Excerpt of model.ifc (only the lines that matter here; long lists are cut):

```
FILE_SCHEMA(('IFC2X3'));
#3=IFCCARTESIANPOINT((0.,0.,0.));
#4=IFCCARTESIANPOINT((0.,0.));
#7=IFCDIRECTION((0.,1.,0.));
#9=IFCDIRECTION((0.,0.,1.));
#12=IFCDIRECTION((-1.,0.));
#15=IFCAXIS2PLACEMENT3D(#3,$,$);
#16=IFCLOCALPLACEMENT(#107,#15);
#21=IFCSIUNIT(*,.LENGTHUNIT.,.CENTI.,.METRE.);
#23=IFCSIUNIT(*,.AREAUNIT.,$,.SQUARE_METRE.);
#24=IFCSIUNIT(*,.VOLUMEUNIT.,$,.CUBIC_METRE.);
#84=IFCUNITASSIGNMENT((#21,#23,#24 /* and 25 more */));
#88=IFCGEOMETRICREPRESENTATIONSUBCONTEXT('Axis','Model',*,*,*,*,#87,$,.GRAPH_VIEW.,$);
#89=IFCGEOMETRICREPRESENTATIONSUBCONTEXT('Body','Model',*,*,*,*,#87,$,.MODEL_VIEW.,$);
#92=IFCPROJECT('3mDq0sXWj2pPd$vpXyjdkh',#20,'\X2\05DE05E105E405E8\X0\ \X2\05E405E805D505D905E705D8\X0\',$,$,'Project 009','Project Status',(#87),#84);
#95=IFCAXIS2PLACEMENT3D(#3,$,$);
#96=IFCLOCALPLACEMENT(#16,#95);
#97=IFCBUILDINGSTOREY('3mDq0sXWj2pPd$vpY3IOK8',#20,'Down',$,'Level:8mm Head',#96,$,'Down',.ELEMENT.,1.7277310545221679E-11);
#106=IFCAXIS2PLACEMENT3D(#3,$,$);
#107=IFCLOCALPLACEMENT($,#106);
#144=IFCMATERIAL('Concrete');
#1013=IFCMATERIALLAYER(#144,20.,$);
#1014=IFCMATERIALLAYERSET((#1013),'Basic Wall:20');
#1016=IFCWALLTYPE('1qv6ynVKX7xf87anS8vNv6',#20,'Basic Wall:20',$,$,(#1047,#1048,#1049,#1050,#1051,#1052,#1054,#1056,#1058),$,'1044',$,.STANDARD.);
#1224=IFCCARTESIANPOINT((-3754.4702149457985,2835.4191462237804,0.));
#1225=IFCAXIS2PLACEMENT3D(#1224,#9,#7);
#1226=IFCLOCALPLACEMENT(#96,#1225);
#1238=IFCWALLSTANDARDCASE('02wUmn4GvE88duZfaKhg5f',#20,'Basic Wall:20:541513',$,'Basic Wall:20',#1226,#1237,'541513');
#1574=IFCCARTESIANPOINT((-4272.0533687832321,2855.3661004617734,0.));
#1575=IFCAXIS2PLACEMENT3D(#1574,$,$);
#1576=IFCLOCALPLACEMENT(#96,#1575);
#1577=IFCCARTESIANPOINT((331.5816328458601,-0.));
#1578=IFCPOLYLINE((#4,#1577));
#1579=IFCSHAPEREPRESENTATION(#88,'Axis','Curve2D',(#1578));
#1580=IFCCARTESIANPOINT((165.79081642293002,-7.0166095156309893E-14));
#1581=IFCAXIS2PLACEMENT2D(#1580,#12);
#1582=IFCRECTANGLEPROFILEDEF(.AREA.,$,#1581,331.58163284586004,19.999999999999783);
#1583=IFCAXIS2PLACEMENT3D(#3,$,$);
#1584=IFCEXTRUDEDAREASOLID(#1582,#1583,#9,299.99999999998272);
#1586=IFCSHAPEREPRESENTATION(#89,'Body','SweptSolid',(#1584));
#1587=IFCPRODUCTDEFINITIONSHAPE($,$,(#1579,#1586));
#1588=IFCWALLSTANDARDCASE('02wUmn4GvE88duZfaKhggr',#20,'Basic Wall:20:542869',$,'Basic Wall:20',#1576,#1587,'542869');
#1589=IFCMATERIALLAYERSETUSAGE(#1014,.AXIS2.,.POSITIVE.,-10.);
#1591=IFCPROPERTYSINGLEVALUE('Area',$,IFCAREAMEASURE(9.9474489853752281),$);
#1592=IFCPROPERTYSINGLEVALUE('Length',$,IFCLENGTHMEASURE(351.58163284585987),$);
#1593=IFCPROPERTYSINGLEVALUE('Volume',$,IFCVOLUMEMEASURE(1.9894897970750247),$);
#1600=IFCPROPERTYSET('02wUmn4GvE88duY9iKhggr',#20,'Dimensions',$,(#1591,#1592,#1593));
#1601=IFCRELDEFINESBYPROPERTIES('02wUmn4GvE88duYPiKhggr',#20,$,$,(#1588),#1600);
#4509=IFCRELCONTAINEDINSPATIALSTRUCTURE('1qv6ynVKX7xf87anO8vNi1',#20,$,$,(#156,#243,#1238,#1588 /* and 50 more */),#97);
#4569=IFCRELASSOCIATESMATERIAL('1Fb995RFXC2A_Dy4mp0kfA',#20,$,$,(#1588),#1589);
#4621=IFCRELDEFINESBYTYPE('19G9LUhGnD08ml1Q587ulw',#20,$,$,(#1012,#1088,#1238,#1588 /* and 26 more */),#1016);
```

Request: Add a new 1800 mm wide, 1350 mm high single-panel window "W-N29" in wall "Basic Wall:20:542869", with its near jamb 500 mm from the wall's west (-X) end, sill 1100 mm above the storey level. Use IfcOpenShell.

```python
import numpy as np
import ifcopenshell
import ifcopenshell.api.feature
import ifcopenshell.api.geometry
import ifcopenshell.api.pset
import ifcopenshell.api.root
import ifcopenshell.api.spatial
import ifcopenshell.api.type
import ifcopenshell.geom
import ifcopenshell.util.element
import ifcopenshell.util.placement
import ifcopenshell.util.representation
import ifcopenshell.util.shape
import ifcopenshell.util.unit

model = ifcopenshell.open("model.ifc")
unit_scale = ifcopenshell.util.unit.calculate_unit_scale(model)
area_scale = ifcopenshell.util.unit.calculate_unit_scale(model, "AREAUNIT")
volume_scale = ifcopenshell.util.unit.calculate_unit_scale(model, "VOLUMEUNIT")
settings = ifcopenshell.geom.settings()


def volume(element):
    """Net volume in cubic metres, openings subtracted."""
    shape = ifcopenshell.geom.create_shape(settings, element)
    return ifcopenshell.util.shape.get_volume(shape.geometry)


wall = model.by_guid("02wUmn4GvE88duZfaKhggr")
storey = ifcopenshell.util.element.get_container(wall, ifc_class="IfcBuildingStorey")
context = ifcopenshell.util.representation.get_context(model, "Model", "Body", "MODEL_VIEW")
before = volume(wall)

width, height, from_end, sill = 1.8, 1.35, 0.5, 1.1  # metres

# The wall runs along its own X axis, and the end named is its -X end.
wall_shape = ifcopenshell.geom.create_shape(settings, wall)
x, y, z = ifcopenshell.util.shape.get_vertices(wall_shape.geometry).T
start = x.min() + from_end
face, thickness = float(y.min()), float(y.max() - y.min())
wall_matrix = ifcopenshell.util.placement.get_local_placement(wall.ObjectPlacement)
level = ifcopenshell.util.placement.get_local_placement(storey.ObjectPlacement)[2, 3]


def in_wall(x, y):
    """Placement at x, y metres in the wall's axes, at sill height."""
    matrix = wall_matrix.copy()
    matrix[:, 3] = wall_matrix @ np.array([x / unit_scale, y / unit_scale, 0.0, 1.0])
    matrix[2, 3] = level + sill / unit_scale
    return matrix


# Opening: a box that overshoots both wall faces by 50 mm.
opening = ifcopenshell.api.root.create_entity(model, ifc_class="IfcOpeningElement")
box = ifcopenshell.api.geometry.add_wall_representation(
    model, context=context, length=width, height=height, thickness=thickness + 0.1
)
ifcopenshell.api.geometry.assign_representation(model, product=opening, representation=box)
ifcopenshell.api.geometry.edit_object_placement(model, product=opening, matrix=in_wall(start, face - 0.05), is_si=False)
ifcopenshell.api.feature.add_feature(model, feature=opening, element=wall)

window = ifcopenshell.api.root.create_entity(model, ifc_class="IfcWindow", name="W-N29")
window.OverallWidth, window.OverallHeight = width / unit_scale, height / unit_scale
body = ifcopenshell.api.geometry.add_window_representation(
    model,
    context=context,
    overall_width=window.OverallWidth,
    overall_height=window.OverallHeight,
    partition_type="SINGLE_PANEL",
)
ifcopenshell.api.geometry.assign_representation(model, product=window, representation=body)
ifcopenshell.api.spatial.assign_container(model, products=[window], relating_structure=storey)
fills = ifcopenshell.api.feature.add_filling(model, opening=opening, element=window)
fills.OwnerHistory = window.OwnerHistory  # required in IFC2X3

# IFC2X3 keeps the operation on the window style.
style = ifcopenshell.api.root.create_entity(model, ifc_class="IfcWindowStyle", name="W-N29")
style.OperationType, style.ConstructionType = "SINGLE_PANEL", "NOTDEFINED"
style.ParameterTakesPrecedence = style.Sizeable = False
ifcopenshell.api.type.assign_type(model, related_objects=[window], relating_type=style)

# Centre the window in the wall's thickness.
ifcopenshell.api.geometry.edit_object_placement(model, product=window, matrix=in_wall(start, face), is_si=False)
window_shape = ifcopenshell.geom.create_shape(settings, window)
depth = ifcopenshell.util.shape.get_vertices(window_shape.geometry)[:, 1]
offset = face + thickness / 2 - (depth.min() + depth.max()) / 2
ifcopenshell.api.geometry.edit_object_placement(model, product=window, matrix=in_wall(start, offset), is_si=False)

after = volume(wall)

# Update the wall's stored quantities.
pset = model.by_id(ifcopenshell.util.element.get_pset(wall, "Dimensions", should_inherit=False)["id"])
ifcopenshell.api.pset.edit_pset(model, pset=pset, properties={
    "Area": model.create_entity("IfcAreaMeasure", after / thickness / area_scale),
    "Volume": model.create_entity("IfcVolumeMeasure", after / volume_scale),
})

print(f"wall volume {before:.3f} -> {after:.3f} m3")

model.write("model_edited.ifc")
```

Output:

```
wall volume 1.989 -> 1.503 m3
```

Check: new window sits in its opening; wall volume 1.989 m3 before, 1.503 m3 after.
